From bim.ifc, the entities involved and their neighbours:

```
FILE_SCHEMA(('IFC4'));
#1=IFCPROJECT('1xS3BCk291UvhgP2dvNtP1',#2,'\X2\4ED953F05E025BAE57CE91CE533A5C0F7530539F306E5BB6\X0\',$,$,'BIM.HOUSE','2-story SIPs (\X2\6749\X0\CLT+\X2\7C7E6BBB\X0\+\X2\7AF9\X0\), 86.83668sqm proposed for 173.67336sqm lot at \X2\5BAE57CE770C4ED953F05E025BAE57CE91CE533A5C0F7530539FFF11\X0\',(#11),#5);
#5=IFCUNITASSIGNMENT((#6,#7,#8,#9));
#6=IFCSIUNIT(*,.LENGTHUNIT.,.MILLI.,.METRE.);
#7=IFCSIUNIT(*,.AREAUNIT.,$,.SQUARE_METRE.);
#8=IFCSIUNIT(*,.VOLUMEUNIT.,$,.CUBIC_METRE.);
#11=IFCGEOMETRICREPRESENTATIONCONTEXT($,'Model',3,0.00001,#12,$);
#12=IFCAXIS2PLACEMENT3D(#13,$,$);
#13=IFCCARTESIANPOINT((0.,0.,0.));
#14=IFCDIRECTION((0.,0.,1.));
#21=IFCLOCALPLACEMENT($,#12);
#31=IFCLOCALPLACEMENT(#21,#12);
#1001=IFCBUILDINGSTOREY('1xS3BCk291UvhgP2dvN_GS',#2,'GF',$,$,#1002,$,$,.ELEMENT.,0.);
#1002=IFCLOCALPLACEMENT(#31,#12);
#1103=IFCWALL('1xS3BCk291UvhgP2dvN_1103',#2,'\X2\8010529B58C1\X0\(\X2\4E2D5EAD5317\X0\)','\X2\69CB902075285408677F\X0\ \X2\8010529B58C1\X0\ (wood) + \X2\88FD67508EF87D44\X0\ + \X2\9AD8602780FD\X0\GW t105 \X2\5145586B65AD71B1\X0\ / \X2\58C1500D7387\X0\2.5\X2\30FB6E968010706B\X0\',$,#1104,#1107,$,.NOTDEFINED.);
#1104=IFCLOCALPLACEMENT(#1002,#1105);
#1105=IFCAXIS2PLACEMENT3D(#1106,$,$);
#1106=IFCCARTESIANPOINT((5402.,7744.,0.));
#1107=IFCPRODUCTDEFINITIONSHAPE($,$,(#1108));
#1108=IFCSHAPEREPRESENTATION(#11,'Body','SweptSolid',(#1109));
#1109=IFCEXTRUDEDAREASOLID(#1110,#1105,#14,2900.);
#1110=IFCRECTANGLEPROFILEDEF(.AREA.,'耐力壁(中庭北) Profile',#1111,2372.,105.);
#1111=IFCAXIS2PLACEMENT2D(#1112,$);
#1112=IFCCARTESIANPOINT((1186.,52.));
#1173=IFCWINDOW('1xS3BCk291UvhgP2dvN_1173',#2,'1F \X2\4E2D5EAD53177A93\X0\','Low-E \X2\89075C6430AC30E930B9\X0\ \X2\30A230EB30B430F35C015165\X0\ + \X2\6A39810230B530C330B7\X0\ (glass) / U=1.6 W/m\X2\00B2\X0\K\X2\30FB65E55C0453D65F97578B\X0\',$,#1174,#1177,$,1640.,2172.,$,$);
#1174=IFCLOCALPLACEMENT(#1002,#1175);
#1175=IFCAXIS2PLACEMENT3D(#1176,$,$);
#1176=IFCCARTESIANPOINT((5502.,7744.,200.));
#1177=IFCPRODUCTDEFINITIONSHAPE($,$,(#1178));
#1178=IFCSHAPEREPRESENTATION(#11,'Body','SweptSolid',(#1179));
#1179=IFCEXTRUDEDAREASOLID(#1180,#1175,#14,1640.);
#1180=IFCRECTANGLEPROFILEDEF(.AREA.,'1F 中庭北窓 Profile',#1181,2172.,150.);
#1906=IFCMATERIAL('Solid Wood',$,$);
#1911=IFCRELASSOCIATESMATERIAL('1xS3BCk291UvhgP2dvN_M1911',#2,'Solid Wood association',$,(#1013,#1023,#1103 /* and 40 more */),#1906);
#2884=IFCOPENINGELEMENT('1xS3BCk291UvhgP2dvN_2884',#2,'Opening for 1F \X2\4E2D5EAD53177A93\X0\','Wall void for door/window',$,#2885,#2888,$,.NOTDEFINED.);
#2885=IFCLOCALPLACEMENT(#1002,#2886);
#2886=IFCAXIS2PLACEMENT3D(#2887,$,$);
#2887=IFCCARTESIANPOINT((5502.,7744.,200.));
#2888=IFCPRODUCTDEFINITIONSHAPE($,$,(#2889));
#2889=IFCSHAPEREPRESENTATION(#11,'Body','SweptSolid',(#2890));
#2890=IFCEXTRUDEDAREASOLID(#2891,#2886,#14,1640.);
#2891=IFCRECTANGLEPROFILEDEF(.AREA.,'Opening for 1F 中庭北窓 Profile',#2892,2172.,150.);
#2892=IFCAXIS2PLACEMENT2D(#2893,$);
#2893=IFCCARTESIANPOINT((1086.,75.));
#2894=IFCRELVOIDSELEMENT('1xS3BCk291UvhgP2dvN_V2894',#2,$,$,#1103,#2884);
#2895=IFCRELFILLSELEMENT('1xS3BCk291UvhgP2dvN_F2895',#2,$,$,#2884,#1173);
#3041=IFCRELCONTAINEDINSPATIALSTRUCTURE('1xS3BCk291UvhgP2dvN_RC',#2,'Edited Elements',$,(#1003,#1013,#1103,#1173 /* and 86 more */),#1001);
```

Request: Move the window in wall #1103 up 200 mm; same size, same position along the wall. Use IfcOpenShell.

```python
import numpy as np
import ifcopenshell
import ifcopenshell.api.geometry
import ifcopenshell.util.placement
import ifcopenshell.util.unit

model = ifcopenshell.open("bim.ifc")
unit_scale = ifcopenshell.util.unit.calculate_unit_scale(model)

window = model.by_guid("1xS3BCk291UvhgP2dvN_1173")
opening = window.FillsVoids[0].RelatingOpeningElement
dz = 0.2 / unit_scale

shift = np.array([0.0, 0.0, dz])
# The window is not placed relative to its opening, so move both.
for product in (opening, window):
    matrix = ifcopenshell.util.placement.get_local_placement(product.ObjectPlacement)
    matrix[:3, 3] += shift
    ifcopenshell.api.geometry.edit_object_placement(model, product=product, matrix=matrix, is_si=False)

print(f"moved by {dz * unit_scale:+.3f} m")

model.write("bim_rev.ifc")
```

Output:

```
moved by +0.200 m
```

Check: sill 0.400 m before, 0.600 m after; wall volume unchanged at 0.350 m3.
